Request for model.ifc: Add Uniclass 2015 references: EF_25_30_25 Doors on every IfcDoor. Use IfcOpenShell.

First a look at what the model holds.

```python
import ifcopenshell

model = ifcopenshell.open("model.ifc")
print(model.schema)
print("classifications:", [c.Name for c in model.by_type("IfcClassification")])
for ifc_class in ("IfcDoor", "IfcRoof", "IfcStair", "IfcWall", "IfcWindow"):
    print(ifc_class, len(model.by_type(ifc_class)))
```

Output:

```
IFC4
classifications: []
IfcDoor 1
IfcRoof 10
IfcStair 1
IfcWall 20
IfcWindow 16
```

```python
import ifcopenshell
import ifcopenshell.api.classification

model = ifcopenshell.open("model.ifc")

system = ifcopenshell.api.classification.add_classification(model, classification="Uniclass 2015")

codes = {
    "IfcDoor": ("EF_25_30_25", "Doors"),
}
for ifc_class, (code, name) in codes.items():
    products = model.by_type(ifc_class)
    ifcopenshell.api.classification.add_reference(
        model, products=products, classification=system, identification=code, name=name
    )
    print(code, len(products))

model.write("model_updated.ifc")
```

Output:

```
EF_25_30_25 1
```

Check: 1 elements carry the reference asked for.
